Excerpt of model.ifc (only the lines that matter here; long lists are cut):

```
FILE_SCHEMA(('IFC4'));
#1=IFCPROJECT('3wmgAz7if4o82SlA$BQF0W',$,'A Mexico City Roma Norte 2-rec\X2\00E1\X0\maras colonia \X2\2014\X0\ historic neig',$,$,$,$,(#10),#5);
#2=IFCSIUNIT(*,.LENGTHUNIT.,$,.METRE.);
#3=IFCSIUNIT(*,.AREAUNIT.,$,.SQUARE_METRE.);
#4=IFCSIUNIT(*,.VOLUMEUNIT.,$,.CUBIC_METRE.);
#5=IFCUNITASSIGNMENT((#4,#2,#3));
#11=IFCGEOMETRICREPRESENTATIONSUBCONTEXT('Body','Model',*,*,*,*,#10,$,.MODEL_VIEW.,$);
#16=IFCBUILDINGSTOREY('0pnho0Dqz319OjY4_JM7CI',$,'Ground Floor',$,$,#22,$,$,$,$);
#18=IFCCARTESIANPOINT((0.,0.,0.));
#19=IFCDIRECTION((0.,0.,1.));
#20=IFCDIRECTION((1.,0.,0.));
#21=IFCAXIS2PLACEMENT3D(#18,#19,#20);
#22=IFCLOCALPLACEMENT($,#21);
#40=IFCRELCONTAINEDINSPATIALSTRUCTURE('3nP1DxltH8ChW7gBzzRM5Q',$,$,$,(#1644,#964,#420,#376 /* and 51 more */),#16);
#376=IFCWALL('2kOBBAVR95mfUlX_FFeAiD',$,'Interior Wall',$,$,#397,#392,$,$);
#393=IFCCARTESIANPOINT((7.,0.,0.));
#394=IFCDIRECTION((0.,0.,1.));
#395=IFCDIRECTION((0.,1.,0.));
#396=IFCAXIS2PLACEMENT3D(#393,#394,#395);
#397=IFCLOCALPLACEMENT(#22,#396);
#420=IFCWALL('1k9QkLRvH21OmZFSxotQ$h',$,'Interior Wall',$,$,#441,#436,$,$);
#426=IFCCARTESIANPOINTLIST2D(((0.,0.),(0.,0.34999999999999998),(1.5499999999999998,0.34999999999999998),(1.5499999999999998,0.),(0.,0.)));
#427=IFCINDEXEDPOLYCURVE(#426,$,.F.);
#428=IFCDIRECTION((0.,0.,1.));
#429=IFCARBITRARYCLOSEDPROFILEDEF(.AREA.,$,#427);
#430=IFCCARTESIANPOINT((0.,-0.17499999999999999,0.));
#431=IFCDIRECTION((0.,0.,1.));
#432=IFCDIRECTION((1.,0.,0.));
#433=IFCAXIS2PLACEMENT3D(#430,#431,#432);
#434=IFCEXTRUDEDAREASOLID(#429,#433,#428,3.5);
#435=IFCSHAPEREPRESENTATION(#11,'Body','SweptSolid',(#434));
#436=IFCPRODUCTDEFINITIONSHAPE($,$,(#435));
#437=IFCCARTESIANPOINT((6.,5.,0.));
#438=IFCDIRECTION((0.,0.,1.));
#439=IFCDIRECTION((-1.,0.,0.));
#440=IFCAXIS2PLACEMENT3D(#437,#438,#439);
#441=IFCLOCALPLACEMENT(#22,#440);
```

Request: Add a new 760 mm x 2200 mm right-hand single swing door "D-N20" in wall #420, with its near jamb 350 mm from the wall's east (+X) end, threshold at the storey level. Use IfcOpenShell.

```python
import numpy as np
import ifcopenshell
import ifcopenshell.api.feature
import ifcopenshell.api.geometry
import ifcopenshell.api.root
import ifcopenshell.api.spatial
import ifcopenshell.geom
import ifcopenshell.util.element
import ifcopenshell.util.placement
import ifcopenshell.util.representation
import ifcopenshell.util.shape
import ifcopenshell.util.unit

model = ifcopenshell.open("model.ifc")
unit_scale = ifcopenshell.util.unit.calculate_unit_scale(model)
settings = ifcopenshell.geom.settings()


def volume(element):
    """Net volume in cubic metres, openings subtracted."""
    shape = ifcopenshell.geom.create_shape(settings, element)
    return ifcopenshell.util.shape.get_volume(shape.geometry)


wall = model.by_guid("1k9QkLRvH21OmZFSxotQ$h")
storey = ifcopenshell.util.element.get_container(wall, ifc_class="IfcBuildingStorey")
context = ifcopenshell.util.representation.get_context(model, "Model", "Body", "MODEL_VIEW")
before = volume(wall)

width, height, from_end, sill = 0.76, 2.2, 0.35, 0.0  # metres

# The wall runs along its own X axis, and the end named is its -X end.
wall_shape = ifcopenshell.geom.create_shape(settings, wall)
x, y, z = ifcopenshell.util.shape.get_vertices(wall_shape.geometry).T
start = x.min() + from_end
face, thickness = float(y.min()), float(y.max() - y.min())
wall_matrix = ifcopenshell.util.placement.get_local_placement(wall.ObjectPlacement)
level = ifcopenshell.util.placement.get_local_placement(storey.ObjectPlacement)[2, 3]


def in_wall(x, y):
    """Placement at x, y metres in the wall's axes, at sill height."""
    matrix = wall_matrix.copy()
    matrix[:, 3] = wall_matrix @ np.array([x / unit_scale, y / unit_scale, 0.0, 1.0])
    matrix[2, 3] = level + sill / unit_scale
    return matrix


# Opening: a box that overshoots both wall faces by 50 mm.
opening = ifcopenshell.api.root.create_entity(model, ifc_class="IfcOpeningElement", predefined_type="OPENING")
box = ifcopenshell.api.geometry.add_wall_representation(
    model, context=context, length=width, height=height, thickness=thickness + 0.1
)
ifcopenshell.api.geometry.assign_representation(model, product=opening, representation=box)
ifcopenshell.api.geometry.edit_object_placement(model, product=opening, matrix=in_wall(start, face - 0.05), is_si=False)
ifcopenshell.api.feature.add_feature(model, feature=opening, element=wall)

door = ifcopenshell.api.root.create_entity(model, ifc_class="IfcDoor", name="D-N20", predefined_type="DOOR")
door.OverallWidth, door.OverallHeight = width / unit_scale, height / unit_scale
door.OperationType = "SINGLE_SWING_RIGHT"
body = ifcopenshell.api.geometry.add_door_representation(
    model,
    context=context,
    overall_width=door.OverallWidth,
    overall_height=door.OverallHeight,
    operation_type="SINGLE_SWING_RIGHT",
    lining_properties={"LiningDepth": thickness / unit_scale, "ThresholdDepth": thickness / unit_scale},
)
ifcopenshell.api.geometry.assign_representation(model, product=door, representation=body)
ifcopenshell.api.spatial.assign_container(model, products=[door], relating_structure=storey)
ifcopenshell.api.feature.add_filling(model, opening=opening, element=door)

# The lining spans the wall, so the door starts at the wall face.
ifcopenshell.api.geometry.edit_object_placement(model, product=door, matrix=in_wall(start, face), is_si=False)

after = volume(wall)

print(f"wall volume {before:.3f} -> {after:.3f} m3")

model.write("model_updated.ifc")
```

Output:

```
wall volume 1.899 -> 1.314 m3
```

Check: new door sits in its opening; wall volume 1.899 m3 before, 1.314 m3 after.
